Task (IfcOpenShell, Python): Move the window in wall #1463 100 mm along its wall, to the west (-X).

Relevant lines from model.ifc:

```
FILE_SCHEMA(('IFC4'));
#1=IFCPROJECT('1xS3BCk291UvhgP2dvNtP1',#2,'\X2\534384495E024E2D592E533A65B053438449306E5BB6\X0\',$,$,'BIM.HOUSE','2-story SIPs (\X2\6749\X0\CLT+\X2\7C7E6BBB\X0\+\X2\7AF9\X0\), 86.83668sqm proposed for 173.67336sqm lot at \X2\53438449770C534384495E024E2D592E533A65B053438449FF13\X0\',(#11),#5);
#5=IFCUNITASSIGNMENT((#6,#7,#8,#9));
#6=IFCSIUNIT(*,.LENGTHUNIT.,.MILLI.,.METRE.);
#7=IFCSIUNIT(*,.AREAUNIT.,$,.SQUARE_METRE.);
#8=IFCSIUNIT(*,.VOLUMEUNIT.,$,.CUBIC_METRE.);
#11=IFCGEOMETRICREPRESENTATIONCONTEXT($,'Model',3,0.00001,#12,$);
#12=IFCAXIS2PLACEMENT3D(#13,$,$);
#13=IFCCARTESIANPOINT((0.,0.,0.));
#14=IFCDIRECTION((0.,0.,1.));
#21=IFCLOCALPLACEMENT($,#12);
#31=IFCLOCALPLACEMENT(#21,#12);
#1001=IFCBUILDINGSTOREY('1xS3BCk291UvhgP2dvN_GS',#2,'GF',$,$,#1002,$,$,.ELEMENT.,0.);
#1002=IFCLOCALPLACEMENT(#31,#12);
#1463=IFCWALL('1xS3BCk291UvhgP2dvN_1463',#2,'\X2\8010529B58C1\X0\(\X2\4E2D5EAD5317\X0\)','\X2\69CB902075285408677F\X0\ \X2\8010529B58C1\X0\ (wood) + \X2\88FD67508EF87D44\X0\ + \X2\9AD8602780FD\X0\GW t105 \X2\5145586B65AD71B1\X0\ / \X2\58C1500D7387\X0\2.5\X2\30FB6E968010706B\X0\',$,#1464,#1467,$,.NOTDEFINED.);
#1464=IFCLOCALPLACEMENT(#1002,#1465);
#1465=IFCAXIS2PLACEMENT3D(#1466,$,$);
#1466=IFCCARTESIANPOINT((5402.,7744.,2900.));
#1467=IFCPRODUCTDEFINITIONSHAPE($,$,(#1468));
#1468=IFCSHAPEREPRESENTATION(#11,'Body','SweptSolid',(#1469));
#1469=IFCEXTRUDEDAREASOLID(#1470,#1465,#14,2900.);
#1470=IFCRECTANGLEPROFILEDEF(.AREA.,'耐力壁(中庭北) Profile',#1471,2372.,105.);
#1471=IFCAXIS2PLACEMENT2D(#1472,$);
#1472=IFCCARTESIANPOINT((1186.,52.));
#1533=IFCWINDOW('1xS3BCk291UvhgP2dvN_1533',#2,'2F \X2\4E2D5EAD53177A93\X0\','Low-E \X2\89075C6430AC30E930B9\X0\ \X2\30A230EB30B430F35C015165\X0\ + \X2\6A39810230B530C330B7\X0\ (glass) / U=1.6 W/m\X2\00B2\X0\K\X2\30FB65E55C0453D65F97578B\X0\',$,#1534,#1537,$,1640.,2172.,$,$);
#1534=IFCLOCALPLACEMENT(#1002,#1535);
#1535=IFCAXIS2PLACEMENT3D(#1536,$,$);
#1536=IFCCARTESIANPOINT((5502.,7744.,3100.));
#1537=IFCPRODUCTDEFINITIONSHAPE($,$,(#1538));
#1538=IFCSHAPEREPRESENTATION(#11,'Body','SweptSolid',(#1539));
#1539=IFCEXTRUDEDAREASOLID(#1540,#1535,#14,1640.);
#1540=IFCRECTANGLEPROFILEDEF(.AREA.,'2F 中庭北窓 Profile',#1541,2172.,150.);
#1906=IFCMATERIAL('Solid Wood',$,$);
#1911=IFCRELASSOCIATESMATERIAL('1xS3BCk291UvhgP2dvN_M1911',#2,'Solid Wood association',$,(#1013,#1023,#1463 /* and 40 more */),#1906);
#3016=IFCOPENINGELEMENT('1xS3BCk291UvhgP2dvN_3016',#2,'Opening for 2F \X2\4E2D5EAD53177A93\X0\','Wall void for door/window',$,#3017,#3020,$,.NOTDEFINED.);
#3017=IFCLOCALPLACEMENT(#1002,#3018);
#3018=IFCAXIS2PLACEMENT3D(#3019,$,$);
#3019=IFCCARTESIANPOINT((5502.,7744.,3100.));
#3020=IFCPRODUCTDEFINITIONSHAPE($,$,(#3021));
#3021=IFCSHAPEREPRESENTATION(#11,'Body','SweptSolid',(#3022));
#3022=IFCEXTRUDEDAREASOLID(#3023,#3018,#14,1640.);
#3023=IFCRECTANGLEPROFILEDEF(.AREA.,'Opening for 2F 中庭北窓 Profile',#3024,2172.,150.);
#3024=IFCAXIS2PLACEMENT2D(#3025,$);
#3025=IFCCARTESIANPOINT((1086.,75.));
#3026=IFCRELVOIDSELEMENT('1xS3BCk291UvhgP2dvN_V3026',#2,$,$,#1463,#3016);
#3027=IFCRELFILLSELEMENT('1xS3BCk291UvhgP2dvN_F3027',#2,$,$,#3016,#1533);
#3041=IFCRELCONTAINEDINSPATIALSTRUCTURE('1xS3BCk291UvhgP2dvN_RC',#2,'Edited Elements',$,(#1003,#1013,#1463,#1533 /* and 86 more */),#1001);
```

```python
import ifcopenshell
import ifcopenshell.api.geometry
import ifcopenshell.util.placement

model = ifcopenshell.open("model.ifc")

window = model.by_id(1533)
opening = window.FillsVoids[0].RelatingOpeningElement
wall = opening.VoidsElements[0].RelatingBuildingElement

wall_matrix = ifcopenshell.util.placement.get_local_placement(wall.ObjectPlacement)
shift = wall_matrix[:3, 0] * -100.0
before = ifcopenshell.util.placement.get_local_placement(window.ObjectPlacement)[:3, 3].copy()

# The window is not placed relative to its opening, so move both.
for product in (opening, window):
    matrix = ifcopenshell.util.placement.get_local_placement(product.ObjectPlacement)
    matrix[:3, 3] += shift
    ifcopenshell.api.geometry.edit_object_placement(model, product=product, matrix=matrix, is_si=False)

after = ifcopenshell.util.placement.get_local_placement(window.ObjectPlacement)[:3, 3]
print("window moved by", (after - before).round(3) + 0.0)

model.write("model_edited.ifc")
```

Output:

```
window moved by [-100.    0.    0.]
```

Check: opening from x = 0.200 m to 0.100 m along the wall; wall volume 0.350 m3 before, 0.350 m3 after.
